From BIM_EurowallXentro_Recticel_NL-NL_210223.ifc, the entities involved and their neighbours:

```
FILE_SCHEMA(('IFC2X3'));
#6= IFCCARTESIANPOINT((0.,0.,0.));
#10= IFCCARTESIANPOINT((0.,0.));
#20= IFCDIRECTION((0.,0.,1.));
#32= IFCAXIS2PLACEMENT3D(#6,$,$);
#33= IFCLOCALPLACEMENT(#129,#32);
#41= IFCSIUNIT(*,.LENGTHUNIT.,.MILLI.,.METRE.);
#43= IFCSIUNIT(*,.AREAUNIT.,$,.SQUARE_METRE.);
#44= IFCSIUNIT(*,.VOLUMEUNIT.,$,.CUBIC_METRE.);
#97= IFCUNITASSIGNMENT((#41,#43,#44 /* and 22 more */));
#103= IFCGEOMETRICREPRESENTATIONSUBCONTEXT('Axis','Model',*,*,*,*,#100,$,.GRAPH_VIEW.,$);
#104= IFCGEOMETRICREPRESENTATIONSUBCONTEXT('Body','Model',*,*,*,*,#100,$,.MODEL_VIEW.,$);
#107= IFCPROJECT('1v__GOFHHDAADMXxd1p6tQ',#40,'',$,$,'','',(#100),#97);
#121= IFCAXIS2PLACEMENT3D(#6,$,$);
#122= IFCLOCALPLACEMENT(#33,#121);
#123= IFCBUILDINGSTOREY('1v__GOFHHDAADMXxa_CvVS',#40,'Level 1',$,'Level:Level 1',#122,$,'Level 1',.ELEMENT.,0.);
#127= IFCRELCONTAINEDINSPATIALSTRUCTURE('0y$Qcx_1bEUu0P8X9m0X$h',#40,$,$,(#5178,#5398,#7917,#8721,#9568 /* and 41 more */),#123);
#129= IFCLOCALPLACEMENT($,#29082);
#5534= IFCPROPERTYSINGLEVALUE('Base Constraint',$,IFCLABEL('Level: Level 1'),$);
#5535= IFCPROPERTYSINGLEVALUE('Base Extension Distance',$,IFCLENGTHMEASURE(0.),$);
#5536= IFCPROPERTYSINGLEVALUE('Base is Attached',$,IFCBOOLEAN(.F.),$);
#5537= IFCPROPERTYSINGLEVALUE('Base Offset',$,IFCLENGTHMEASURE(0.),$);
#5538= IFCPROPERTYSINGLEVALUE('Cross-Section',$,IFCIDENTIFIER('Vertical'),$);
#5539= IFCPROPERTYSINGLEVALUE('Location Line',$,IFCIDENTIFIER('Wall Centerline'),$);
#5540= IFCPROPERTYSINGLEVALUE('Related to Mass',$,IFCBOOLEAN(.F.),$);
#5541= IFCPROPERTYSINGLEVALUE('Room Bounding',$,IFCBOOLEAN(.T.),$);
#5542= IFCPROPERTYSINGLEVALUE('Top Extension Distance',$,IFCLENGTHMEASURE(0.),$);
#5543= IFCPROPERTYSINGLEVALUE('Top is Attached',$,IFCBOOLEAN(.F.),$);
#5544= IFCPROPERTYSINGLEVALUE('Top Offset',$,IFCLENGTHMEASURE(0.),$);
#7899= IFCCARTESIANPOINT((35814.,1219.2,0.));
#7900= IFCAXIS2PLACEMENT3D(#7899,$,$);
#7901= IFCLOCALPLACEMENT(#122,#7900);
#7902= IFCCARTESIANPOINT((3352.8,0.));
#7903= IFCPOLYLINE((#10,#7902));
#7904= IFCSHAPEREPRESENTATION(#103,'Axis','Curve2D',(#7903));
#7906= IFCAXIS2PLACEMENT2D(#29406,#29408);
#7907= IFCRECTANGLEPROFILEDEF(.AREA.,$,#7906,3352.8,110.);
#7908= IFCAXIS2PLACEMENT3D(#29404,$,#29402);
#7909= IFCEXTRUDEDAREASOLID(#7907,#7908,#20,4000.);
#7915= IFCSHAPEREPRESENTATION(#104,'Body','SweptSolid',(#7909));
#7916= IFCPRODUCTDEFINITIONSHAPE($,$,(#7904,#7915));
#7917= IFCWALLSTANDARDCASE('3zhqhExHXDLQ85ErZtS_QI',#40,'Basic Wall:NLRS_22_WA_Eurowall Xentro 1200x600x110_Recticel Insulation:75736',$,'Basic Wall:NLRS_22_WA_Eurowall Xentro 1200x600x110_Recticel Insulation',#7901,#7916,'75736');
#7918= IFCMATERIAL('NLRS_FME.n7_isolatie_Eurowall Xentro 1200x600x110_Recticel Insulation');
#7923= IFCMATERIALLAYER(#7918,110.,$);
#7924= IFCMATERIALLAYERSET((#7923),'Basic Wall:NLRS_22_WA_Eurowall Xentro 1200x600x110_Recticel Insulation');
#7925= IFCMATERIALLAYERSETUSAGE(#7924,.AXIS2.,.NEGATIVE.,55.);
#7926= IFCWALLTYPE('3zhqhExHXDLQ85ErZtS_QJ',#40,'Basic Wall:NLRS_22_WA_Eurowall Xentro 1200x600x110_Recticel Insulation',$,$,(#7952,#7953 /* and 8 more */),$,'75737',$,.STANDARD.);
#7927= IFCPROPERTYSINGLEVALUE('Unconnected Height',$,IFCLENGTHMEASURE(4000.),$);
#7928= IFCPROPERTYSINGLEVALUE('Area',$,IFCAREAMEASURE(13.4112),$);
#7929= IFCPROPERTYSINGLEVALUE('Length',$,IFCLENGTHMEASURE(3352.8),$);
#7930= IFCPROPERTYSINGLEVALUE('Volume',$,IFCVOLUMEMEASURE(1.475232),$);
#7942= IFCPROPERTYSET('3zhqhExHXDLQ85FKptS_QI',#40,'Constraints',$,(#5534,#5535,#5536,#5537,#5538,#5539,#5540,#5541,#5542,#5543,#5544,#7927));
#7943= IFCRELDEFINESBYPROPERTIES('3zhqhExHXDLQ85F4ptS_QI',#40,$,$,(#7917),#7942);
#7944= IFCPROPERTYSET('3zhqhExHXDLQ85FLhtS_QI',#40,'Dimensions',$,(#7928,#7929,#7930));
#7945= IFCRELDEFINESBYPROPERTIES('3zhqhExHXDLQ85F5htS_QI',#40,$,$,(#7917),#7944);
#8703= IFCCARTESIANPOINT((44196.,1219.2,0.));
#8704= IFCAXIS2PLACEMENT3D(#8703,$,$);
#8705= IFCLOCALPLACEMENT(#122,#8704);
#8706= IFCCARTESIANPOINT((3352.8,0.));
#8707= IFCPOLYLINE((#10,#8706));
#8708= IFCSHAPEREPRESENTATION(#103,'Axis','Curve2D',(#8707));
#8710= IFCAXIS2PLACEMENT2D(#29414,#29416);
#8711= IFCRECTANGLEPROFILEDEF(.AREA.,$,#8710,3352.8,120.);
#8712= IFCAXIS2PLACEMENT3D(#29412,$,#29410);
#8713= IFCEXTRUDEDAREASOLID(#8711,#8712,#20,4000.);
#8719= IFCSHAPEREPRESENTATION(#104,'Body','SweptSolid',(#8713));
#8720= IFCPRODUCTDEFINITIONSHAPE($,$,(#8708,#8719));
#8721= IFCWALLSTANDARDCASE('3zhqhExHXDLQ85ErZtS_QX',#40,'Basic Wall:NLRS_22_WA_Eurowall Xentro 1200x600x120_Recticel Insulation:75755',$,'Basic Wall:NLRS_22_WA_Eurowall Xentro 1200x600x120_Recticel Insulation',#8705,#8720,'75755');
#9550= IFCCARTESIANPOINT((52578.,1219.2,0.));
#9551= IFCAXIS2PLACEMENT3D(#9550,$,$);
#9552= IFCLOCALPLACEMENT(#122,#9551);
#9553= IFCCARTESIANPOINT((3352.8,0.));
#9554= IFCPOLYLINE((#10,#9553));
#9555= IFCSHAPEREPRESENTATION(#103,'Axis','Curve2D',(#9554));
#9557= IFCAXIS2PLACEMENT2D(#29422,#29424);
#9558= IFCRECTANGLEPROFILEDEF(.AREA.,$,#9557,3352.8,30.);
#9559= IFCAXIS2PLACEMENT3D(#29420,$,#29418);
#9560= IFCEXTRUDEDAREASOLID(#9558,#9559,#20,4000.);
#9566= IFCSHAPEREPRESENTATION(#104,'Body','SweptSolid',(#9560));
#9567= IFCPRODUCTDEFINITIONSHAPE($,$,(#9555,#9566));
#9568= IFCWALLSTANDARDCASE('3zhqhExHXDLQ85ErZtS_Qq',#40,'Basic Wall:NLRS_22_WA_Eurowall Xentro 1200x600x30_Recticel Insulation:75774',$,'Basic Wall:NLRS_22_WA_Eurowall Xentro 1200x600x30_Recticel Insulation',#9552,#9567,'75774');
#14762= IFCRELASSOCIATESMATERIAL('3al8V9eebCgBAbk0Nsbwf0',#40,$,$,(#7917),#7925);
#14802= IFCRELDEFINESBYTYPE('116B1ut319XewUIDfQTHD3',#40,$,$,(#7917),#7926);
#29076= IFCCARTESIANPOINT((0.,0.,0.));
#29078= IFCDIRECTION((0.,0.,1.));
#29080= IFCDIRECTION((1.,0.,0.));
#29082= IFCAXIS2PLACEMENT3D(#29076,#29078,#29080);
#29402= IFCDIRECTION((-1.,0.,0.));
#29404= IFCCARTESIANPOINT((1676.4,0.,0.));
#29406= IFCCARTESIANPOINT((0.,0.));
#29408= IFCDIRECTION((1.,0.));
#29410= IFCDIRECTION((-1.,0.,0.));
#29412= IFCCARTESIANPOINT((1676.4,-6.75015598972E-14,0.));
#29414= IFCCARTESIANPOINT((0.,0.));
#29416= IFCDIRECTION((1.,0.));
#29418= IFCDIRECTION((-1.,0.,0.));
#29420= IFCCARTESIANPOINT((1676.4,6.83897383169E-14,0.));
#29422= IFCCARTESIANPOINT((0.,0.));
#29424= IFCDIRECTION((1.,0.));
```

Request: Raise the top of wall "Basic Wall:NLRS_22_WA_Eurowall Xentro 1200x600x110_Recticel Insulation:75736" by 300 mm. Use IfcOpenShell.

```python
import ifcopenshell
import ifcopenshell.api.pset
import ifcopenshell.geom
import ifcopenshell.util.element
import ifcopenshell.util.representation
import ifcopenshell.util.shape
import ifcopenshell.util.unit

model = ifcopenshell.open("BIM_EurowallXentro_Recticel_NL-NL_210223.ifc")
area_scale = ifcopenshell.util.unit.calculate_unit_scale(model, "AREAUNIT")
volume_scale = ifcopenshell.util.unit.calculate_unit_scale(model, "VOLUMEUNIT")
settings = ifcopenshell.geom.settings()


def volume(element):
    """Net volume in cubic metres, openings subtracted."""
    shape = ifcopenshell.geom.create_shape(settings, element)
    return ifcopenshell.util.shape.get_volume(shape.geometry)


wall = model.by_guid("3zhqhExHXDLQ85ErZtS_QI")
before = volume(wall)

body = ifcopenshell.util.representation.get_representation(wall, "Model", "Body")
solid = body.Items[0]
old_height = solid.Depth
solid.Depth += 300.0
after = volume(wall)
thickness = 0.11  # wall thickness in metres

# Update the stored height, areas and volumes.
pset = model.by_id(ifcopenshell.util.element.get_pset(wall, "Constraints", should_inherit=False)["id"])
ifcopenshell.api.pset.edit_pset(model, pset=pset, properties={
    "Unconnected Height": model.create_entity("IfcLengthMeasure", solid.Depth),
})
pset = model.by_id(ifcopenshell.util.element.get_pset(wall, "Dimensions", should_inherit=False)["id"])
ifcopenshell.api.pset.edit_pset(model, pset=pset, properties={
    "Area": model.create_entity("IfcAreaMeasure", after / thickness / area_scale),
    "Volume": model.create_entity("IfcVolumeMeasure", after / volume_scale),
})

print(f"height {old_height:g} -> {solid.Depth:g}, volume {before:.3f} -> {after:.3f} m3")

model.write("BIM_EurowallXentro_Recticel_NL-NL_210223-out.ifc")
```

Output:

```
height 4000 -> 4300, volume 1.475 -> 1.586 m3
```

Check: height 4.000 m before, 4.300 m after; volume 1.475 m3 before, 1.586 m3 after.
